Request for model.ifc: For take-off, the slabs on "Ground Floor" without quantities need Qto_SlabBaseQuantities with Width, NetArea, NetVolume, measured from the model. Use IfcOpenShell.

First a look at what the model holds.

```python
import ifcopenshell
import ifcopenshell.util.element
import ifcopenshell.util.unit

model = ifcopenshell.open("model.ifc")
print(model.schema)
for unit_type in ("LENGTHUNIT", "AREAUNIT", "VOLUMEUNIT"):
    print(unit_type, ifcopenshell.util.unit.calculate_unit_scale(model, unit_type))
storey = next(s for s in model.by_type("IfcBuildingStorey") if s.Name == "Ground Floor")
slabs = [e for e in ifcopenshell.util.element.get_decomposition(storey) if e.is_a("IfcSlab")]
for e in sorted(slabs, key=lambda e: e.id()):
    print(e.id(), e.is_a(), e.Name, list(ifcopenshell.util.element.get_psets(e, qtos_only=True)), sep=" | ")
```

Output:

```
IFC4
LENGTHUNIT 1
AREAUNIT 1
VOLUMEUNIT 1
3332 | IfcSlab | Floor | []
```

```python
import ifcopenshell
import ifcopenshell.api.pset
import ifcopenshell.geom
import ifcopenshell.util.element
import ifcopenshell.util.shape
import ifcopenshell.util.unit

model = ifcopenshell.open("model.ifc")
unit_scale = ifcopenshell.util.unit.calculate_unit_scale(model)
area_scale = ifcopenshell.util.unit.calculate_unit_scale(model, "AREAUNIT")
volume_scale = ifcopenshell.util.unit.calculate_unit_scale(model, "VOLUMEUNIT")
settings = ifcopenshell.geom.settings()

storey = next(s for s in model.by_type("IfcBuildingStorey") if s.Name == "Ground Floor")
slabs = [e for e in ifcopenshell.util.element.get_decomposition(storey) if e.is_a("IfcSlab")]

for e in sorted(slabs, key=lambda e: e.id()):
    if ifcopenshell.util.element.get_psets(e, qtos_only=True, should_inherit=False):
        continue
    # Geometry comes back in metres, in the element's own axes.
    shape = ifcopenshell.geom.create_shape(settings, e)
    values = {
        "Width": ifcopenshell.util.shape.get_z(shape.geometry) / unit_scale,
        "NetArea": ifcopenshell.util.shape.get_footprint_area(shape.geometry) / area_scale,
        "NetVolume": ifcopenshell.util.shape.get_volume(shape.geometry) / volume_scale,
    }
    qto = ifcopenshell.api.pset.add_qto(model, product=e, name="Qto_SlabBaseQuantities")
    ifcopenshell.api.pset.edit_qto(model, qto=qto, properties=values)
    print(e.id(), {k: round(v, 3) for k, v in values.items()})

model.write("model_edited.ifc")
```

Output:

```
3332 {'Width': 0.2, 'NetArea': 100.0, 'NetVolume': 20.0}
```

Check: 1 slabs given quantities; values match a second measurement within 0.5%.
